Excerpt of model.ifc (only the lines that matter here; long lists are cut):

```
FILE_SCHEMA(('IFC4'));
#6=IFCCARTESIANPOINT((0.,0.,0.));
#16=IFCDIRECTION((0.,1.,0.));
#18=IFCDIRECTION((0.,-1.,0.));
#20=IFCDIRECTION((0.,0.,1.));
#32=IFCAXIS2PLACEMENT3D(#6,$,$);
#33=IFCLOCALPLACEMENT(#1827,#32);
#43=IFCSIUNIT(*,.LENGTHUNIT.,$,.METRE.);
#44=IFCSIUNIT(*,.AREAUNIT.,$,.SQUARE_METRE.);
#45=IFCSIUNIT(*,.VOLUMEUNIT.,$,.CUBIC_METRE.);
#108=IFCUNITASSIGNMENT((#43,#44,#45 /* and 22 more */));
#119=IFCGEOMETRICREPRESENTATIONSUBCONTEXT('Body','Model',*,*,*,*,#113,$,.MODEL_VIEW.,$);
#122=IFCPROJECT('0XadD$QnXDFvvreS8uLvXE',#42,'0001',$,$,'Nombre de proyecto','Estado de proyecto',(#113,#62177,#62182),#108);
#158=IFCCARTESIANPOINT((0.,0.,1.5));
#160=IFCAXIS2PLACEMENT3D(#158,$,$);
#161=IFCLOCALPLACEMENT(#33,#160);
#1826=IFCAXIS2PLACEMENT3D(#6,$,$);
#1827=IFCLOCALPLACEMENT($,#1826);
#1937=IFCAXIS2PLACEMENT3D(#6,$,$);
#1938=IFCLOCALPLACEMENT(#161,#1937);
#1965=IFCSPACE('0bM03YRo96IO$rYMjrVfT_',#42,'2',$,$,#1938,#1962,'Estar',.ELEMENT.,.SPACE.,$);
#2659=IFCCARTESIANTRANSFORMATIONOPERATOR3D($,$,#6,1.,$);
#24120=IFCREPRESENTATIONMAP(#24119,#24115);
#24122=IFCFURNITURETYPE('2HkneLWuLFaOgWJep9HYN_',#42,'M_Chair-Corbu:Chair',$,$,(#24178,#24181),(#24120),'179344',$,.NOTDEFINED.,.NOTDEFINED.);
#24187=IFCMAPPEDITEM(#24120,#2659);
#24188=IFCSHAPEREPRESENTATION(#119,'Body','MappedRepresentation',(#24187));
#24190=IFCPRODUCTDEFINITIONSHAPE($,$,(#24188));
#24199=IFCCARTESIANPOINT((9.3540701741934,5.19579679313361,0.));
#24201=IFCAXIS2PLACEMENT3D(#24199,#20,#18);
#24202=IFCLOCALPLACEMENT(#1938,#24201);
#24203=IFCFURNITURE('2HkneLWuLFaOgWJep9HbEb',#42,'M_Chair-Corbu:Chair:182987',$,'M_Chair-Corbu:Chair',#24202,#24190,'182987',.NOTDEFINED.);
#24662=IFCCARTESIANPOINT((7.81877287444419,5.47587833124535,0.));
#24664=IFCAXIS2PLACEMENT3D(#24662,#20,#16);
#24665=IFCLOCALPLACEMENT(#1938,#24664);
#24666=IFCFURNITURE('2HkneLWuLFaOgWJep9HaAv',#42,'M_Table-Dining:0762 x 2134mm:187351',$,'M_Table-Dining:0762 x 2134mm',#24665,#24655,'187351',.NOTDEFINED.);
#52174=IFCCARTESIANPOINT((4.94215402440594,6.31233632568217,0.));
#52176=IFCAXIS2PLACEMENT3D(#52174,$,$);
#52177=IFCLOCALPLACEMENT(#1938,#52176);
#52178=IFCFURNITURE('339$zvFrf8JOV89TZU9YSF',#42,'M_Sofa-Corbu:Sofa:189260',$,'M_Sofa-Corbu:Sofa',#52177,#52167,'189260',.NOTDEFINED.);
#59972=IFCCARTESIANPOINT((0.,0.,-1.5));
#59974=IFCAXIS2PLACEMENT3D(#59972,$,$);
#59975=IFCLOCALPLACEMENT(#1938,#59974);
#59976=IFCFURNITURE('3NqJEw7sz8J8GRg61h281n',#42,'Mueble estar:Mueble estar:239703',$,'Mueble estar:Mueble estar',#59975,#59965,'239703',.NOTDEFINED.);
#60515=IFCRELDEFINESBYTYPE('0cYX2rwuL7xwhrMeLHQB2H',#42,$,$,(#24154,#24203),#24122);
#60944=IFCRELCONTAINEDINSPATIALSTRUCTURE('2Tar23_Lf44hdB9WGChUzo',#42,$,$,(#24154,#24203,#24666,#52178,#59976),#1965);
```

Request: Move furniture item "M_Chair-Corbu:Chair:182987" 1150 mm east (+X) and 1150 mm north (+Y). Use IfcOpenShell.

```python
import ifcopenshell
import ifcopenshell.api.geometry
import ifcopenshell.util.placement
import ifcopenshell.util.unit

model = ifcopenshell.open("model.ifc")
unit_scale = ifcopenshell.util.unit.calculate_unit_scale(model)

item = model.by_guid("2HkneLWuLFaOgWJep9HbEb")
matrix = ifcopenshell.util.placement.get_local_placement(item.ObjectPlacement)
matrix[0, 3] += 1.15 / unit_scale
matrix[1, 3] += 1.15 / unit_scale
ifcopenshell.api.geometry.edit_object_placement(model, product=item, matrix=matrix, is_si=False)

print(ifcopenshell.util.placement.get_local_placement(item.ObjectPlacement).round(3) + 0.0)

model.write("model_rev.ifc")
```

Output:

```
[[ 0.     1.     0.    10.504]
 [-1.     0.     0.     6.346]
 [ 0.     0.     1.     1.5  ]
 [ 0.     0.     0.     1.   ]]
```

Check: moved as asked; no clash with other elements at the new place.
